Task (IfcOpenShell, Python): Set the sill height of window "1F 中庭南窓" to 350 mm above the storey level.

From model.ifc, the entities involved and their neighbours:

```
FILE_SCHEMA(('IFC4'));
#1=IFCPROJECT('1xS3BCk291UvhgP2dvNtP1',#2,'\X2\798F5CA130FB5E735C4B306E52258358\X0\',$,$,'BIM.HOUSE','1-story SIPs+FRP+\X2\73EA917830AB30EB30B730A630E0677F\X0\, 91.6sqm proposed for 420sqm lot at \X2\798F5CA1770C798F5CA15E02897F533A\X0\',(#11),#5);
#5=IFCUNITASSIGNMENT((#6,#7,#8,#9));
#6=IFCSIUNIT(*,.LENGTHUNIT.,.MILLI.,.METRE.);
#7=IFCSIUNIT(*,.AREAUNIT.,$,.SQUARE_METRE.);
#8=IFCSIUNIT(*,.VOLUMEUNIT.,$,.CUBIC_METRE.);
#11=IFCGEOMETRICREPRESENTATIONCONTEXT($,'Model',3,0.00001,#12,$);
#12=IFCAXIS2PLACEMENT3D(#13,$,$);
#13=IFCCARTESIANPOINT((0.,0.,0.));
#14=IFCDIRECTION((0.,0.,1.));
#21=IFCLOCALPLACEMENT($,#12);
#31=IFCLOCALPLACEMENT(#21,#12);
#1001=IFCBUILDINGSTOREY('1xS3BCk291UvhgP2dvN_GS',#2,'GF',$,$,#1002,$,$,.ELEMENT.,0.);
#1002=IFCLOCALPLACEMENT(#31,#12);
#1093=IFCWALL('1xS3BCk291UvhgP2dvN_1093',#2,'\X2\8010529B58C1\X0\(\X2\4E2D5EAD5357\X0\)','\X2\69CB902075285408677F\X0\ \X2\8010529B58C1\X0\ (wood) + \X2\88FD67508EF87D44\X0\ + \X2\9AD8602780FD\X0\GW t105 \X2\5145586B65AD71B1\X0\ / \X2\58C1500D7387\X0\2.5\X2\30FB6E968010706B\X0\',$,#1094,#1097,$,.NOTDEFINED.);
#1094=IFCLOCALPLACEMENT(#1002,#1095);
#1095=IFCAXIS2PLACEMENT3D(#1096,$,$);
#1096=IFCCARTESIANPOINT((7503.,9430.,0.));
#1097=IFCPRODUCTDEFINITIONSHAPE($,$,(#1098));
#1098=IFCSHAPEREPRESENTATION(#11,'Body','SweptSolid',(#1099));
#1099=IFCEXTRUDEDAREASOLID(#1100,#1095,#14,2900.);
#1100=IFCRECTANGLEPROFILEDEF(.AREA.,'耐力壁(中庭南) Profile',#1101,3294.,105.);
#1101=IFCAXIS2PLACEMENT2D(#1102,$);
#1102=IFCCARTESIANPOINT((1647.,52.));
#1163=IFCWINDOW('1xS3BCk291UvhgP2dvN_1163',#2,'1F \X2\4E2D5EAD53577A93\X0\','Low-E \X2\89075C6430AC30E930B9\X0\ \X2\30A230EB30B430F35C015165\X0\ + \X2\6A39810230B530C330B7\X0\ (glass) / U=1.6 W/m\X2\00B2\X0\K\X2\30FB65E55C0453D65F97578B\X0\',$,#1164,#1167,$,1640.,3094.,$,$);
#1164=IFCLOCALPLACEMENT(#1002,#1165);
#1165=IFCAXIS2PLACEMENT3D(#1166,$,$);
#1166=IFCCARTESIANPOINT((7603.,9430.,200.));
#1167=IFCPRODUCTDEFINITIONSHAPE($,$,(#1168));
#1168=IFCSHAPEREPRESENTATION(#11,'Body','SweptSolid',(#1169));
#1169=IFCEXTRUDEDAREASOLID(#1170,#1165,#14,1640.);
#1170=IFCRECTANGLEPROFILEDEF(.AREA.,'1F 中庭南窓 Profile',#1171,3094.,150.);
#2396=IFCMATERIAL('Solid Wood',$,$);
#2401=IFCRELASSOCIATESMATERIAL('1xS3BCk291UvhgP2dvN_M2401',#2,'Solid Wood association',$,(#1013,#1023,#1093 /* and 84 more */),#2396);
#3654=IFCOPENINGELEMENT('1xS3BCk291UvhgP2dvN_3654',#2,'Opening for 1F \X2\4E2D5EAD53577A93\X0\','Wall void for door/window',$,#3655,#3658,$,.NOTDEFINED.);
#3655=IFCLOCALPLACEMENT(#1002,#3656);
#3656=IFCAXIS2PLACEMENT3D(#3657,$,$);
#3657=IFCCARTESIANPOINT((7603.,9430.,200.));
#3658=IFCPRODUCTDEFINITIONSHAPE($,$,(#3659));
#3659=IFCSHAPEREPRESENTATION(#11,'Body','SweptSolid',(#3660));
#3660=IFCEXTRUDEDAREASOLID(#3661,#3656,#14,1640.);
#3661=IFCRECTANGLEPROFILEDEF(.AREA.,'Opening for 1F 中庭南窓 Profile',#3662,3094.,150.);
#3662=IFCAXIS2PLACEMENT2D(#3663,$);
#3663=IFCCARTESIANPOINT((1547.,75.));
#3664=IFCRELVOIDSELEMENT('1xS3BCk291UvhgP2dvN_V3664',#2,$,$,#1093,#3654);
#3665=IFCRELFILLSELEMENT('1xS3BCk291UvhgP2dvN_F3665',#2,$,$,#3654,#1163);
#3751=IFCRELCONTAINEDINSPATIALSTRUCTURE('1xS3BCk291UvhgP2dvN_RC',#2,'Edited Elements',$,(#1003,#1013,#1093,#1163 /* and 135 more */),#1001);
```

```python
import numpy as np
import ifcopenshell
import ifcopenshell.api.geometry
import ifcopenshell.geom
import ifcopenshell.util.element
import ifcopenshell.util.placement
import ifcopenshell.util.shape
import ifcopenshell.util.unit

model = ifcopenshell.open("model.ifc")
unit_scale = ifcopenshell.util.unit.calculate_unit_scale(model)

window = model.by_guid("1xS3BCk291UvhgP2dvN_1163")
opening = window.FillsVoids[0].RelatingOpeningElement
storey = ifcopenshell.util.element.get_container(window, ifc_class="IfcBuildingStorey")
level = ifcopenshell.util.placement.get_local_placement(storey.ObjectPlacement)[2, 3]

# The opening's origin need not be at the sill, so measure its lowest point.
shape = ifcopenshell.geom.create_shape(ifcopenshell.geom.settings(), opening)
bottom = ifcopenshell.util.shape.get_shape_bottom_elevation(shape, shape.geometry) / unit_scale
dz = level + 0.35 / unit_scale - bottom

shift = np.array([0.0, 0.0, dz])
# The window is not placed relative to its opening, so move both.
for product in (opening, window):
    matrix = ifcopenshell.util.placement.get_local_placement(product.ObjectPlacement)
    matrix[:3, 3] += shift
    ifcopenshell.api.geometry.edit_object_placement(model, product=product, matrix=matrix, is_si=False)

print(f"moved by {dz * unit_scale:+.3f} m")

model.write("model-out.ifc")
```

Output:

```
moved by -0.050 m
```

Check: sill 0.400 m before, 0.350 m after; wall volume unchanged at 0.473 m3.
